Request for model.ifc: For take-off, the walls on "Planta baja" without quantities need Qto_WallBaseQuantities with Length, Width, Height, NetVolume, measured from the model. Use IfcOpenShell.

First a look at what the model holds.

```python
import ifcopenshell
import ifcopenshell.util.element
import ifcopenshell.util.unit

model = ifcopenshell.open("model.ifc")
print(model.schema)
for unit_type in ("LENGTHUNIT", "AREAUNIT", "VOLUMEUNIT"):
    print(unit_type, ifcopenshell.util.unit.calculate_unit_scale(model, unit_type))
storey = next(s for s in model.by_type("IfcBuildingStorey") if s.Name == "Planta baja")
walls = [e for e in ifcopenshell.util.element.get_decomposition(storey) if e.is_a("IfcWall")]
for e in sorted(walls, key=lambda e: e.id()):
    print(e.id(), e.is_a(), e.Name, list(ifcopenshell.util.element.get_psets(e, qtos_only=True)), sep=" | ")
```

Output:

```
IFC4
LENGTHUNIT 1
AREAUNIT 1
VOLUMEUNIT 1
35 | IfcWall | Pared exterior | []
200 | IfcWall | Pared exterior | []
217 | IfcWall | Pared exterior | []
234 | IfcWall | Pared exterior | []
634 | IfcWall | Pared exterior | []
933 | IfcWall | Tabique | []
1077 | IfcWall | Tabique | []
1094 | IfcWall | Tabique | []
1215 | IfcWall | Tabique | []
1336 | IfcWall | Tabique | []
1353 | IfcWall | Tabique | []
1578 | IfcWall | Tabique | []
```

```python
import ifcopenshell
import ifcopenshell.api.pset
import ifcopenshell.geom
import ifcopenshell.util.element
import ifcopenshell.util.shape
import ifcopenshell.util.unit

model = ifcopenshell.open("model.ifc")
unit_scale = ifcopenshell.util.unit.calculate_unit_scale(model)
volume_scale = ifcopenshell.util.unit.calculate_unit_scale(model, "VOLUMEUNIT")
settings = ifcopenshell.geom.settings()

storey = next(s for s in model.by_type("IfcBuildingStorey") if s.Name == "Planta baja")
walls = [e for e in ifcopenshell.util.element.get_decomposition(storey) if e.is_a("IfcWall")]

for e in sorted(walls, key=lambda e: e.id()):
    if ifcopenshell.util.element.get_psets(e, qtos_only=True, should_inherit=False):
        continue
    # Geometry comes back in metres, in the element's own axes.
    shape = ifcopenshell.geom.create_shape(settings, e)
    values = {
        "Length": ifcopenshell.util.shape.get_x(shape.geometry) / unit_scale,
        "Width": ifcopenshell.util.shape.get_y(shape.geometry) / unit_scale,
        "Height": ifcopenshell.util.shape.get_z(shape.geometry) / unit_scale,
        "NetVolume": ifcopenshell.util.shape.get_volume(shape.geometry) / volume_scale,
    }
    qto = ifcopenshell.api.pset.add_qto(model, product=e, name="Qto_WallBaseQuantities")
    ifcopenshell.api.pset.edit_qto(model, qto=qto, properties=values)
    print(e.id(), {k: round(v, 3) for k, v in values.items()})

model.write("model_v2.ifc")
```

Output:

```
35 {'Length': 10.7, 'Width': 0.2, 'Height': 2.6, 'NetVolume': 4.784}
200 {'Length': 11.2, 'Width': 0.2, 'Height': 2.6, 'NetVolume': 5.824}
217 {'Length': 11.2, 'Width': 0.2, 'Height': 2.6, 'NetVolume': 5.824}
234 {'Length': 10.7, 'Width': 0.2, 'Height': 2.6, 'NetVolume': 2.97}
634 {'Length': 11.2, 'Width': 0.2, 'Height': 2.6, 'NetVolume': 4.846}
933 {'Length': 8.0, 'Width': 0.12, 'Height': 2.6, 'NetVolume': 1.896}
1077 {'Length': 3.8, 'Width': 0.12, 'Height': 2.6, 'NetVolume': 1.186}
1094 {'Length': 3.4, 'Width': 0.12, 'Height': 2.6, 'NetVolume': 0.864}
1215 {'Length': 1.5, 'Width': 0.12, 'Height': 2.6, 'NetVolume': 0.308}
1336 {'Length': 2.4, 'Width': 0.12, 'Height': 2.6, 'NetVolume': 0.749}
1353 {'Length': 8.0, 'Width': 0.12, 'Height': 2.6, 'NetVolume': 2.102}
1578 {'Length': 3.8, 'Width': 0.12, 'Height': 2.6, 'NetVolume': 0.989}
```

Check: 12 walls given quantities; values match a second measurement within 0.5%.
